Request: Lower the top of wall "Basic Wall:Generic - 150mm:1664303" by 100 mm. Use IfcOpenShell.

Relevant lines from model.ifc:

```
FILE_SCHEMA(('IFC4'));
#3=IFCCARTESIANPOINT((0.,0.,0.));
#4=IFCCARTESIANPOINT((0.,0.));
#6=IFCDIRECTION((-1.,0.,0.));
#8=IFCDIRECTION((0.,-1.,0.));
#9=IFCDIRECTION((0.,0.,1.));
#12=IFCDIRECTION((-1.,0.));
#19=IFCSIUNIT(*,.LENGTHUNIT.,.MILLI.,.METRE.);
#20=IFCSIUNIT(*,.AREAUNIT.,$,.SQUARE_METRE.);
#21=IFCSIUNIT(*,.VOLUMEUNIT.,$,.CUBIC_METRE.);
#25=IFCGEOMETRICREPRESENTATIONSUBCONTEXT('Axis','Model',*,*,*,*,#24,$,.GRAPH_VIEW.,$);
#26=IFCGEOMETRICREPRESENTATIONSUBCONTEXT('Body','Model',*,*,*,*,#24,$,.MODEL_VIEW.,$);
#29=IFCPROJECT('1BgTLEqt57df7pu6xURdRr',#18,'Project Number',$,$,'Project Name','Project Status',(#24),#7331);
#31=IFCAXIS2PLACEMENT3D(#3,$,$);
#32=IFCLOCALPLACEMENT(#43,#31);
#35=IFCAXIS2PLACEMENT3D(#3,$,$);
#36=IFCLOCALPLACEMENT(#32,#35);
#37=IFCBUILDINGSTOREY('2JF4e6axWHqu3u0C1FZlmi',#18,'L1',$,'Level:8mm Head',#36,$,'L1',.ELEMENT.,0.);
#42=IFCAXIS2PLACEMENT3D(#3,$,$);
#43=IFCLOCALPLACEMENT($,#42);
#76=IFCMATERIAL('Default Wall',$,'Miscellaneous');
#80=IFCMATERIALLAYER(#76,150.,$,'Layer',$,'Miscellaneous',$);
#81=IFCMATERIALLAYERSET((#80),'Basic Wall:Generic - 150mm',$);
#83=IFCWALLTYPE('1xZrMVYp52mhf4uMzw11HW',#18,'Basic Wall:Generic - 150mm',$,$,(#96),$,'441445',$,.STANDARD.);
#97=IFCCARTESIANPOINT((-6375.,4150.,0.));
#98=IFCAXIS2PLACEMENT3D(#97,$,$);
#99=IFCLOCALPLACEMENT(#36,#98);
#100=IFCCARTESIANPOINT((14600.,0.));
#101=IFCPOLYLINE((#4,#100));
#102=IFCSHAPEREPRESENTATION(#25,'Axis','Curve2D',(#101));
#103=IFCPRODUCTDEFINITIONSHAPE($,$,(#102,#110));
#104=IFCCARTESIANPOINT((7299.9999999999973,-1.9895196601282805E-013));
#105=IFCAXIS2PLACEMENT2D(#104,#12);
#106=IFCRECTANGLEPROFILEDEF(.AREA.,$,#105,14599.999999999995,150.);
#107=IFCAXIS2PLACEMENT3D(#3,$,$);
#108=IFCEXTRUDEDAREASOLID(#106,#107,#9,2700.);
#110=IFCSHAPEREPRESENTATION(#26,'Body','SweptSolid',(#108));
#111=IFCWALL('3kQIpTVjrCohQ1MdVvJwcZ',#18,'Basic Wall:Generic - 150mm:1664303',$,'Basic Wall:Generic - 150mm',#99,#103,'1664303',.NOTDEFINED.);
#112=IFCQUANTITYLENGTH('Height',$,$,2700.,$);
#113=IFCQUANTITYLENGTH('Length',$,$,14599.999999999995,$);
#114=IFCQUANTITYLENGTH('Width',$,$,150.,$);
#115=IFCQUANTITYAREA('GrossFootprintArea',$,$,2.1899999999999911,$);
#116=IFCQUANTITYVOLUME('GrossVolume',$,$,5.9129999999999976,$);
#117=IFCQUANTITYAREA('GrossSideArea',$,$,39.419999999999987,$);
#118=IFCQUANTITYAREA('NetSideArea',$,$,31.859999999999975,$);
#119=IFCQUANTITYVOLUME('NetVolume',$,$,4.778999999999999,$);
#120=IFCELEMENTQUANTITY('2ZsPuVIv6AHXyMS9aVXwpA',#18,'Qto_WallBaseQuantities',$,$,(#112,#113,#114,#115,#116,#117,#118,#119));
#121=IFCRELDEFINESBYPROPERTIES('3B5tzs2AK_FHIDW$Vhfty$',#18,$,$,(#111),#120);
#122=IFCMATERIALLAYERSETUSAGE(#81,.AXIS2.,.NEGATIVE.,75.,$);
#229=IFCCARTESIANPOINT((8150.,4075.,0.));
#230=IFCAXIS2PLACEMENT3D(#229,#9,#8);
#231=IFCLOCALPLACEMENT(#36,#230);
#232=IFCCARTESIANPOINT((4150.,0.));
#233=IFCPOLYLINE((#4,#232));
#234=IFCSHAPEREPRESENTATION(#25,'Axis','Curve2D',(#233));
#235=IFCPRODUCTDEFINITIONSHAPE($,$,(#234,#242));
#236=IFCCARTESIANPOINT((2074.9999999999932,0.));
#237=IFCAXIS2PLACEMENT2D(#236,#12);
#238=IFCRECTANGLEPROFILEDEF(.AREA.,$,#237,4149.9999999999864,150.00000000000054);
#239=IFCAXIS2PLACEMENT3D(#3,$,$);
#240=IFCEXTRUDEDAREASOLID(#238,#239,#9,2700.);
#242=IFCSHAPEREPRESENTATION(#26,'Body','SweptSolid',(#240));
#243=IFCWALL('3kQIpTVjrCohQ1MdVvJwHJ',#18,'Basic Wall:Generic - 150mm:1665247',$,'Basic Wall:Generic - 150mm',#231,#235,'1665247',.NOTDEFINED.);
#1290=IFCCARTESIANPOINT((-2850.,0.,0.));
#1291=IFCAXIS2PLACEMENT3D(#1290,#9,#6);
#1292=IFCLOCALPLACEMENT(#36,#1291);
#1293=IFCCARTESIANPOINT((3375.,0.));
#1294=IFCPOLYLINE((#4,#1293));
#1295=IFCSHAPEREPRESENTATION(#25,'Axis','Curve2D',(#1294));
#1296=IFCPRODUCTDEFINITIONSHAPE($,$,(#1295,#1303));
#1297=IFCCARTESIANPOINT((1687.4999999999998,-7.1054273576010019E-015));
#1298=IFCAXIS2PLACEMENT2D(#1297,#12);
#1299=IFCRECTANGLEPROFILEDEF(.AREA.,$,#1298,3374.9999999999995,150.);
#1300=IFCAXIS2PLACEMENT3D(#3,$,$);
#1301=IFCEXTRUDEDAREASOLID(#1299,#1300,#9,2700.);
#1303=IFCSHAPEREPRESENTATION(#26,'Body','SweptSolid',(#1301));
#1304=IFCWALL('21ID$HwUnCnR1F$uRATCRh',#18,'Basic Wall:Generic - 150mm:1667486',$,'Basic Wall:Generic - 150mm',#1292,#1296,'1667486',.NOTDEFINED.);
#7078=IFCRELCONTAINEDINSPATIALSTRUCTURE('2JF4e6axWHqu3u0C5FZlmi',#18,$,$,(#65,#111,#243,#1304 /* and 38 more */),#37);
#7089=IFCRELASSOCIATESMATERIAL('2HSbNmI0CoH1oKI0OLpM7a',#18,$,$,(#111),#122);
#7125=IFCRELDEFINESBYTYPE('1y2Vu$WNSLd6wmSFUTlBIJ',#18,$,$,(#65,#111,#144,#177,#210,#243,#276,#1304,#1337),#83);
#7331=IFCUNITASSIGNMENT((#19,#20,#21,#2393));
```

```python
import ifcopenshell
import ifcopenshell.api.pset
import ifcopenshell.geom
import ifcopenshell.util.element
import ifcopenshell.util.representation
import ifcopenshell.util.shape
import ifcopenshell.util.unit

model = ifcopenshell.open("model.ifc")
unit_scale = ifcopenshell.util.unit.calculate_unit_scale(model)
area_scale = ifcopenshell.util.unit.calculate_unit_scale(model, "AREAUNIT")
volume_scale = ifcopenshell.util.unit.calculate_unit_scale(model, "VOLUMEUNIT")
settings = ifcopenshell.geom.settings()


def volume(element):
    """Net volume in cubic metres, openings subtracted."""
    shape = ifcopenshell.geom.create_shape(settings, element)
    return ifcopenshell.util.shape.get_volume(shape.geometry)


wall = model.by_guid("3kQIpTVjrCohQ1MdVvJwcZ")
before = volume(wall)

body = ifcopenshell.util.representation.get_representation(wall, "Model", "Body")
solid = body.Items[0]
old_height = solid.Depth
solid.Depth -= 100.0
after = volume(wall)
thickness = 0.15  # wall thickness in metres

# Update the stored height, areas and volumes.
qto = model.by_id(ifcopenshell.util.element.get_pset(wall, "Qto_WallBaseQuantities", should_inherit=False)["id"])
ifcopenshell.api.pset.edit_qto(model, qto=qto, properties={
    "Height": solid.Depth,
    "GrossVolume": ifcopenshell.util.element.get_pset(wall, "Qto_WallBaseQuantities", "GrossVolume") * solid.Depth / old_height,
    "GrossSideArea": ifcopenshell.util.element.get_pset(wall, "Qto_WallBaseQuantities", "GrossSideArea") * solid.Depth / old_height,
    "NetSideArea": after / thickness / area_scale,
    "NetVolume": after / volume_scale,
})

print(f"height {old_height:g} -> {solid.Depth:g}, volume {before:.3f} -> {after:.3f} m3")

model.write("model_rev.ifc")
```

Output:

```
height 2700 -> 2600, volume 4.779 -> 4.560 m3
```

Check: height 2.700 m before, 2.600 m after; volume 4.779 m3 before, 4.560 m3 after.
